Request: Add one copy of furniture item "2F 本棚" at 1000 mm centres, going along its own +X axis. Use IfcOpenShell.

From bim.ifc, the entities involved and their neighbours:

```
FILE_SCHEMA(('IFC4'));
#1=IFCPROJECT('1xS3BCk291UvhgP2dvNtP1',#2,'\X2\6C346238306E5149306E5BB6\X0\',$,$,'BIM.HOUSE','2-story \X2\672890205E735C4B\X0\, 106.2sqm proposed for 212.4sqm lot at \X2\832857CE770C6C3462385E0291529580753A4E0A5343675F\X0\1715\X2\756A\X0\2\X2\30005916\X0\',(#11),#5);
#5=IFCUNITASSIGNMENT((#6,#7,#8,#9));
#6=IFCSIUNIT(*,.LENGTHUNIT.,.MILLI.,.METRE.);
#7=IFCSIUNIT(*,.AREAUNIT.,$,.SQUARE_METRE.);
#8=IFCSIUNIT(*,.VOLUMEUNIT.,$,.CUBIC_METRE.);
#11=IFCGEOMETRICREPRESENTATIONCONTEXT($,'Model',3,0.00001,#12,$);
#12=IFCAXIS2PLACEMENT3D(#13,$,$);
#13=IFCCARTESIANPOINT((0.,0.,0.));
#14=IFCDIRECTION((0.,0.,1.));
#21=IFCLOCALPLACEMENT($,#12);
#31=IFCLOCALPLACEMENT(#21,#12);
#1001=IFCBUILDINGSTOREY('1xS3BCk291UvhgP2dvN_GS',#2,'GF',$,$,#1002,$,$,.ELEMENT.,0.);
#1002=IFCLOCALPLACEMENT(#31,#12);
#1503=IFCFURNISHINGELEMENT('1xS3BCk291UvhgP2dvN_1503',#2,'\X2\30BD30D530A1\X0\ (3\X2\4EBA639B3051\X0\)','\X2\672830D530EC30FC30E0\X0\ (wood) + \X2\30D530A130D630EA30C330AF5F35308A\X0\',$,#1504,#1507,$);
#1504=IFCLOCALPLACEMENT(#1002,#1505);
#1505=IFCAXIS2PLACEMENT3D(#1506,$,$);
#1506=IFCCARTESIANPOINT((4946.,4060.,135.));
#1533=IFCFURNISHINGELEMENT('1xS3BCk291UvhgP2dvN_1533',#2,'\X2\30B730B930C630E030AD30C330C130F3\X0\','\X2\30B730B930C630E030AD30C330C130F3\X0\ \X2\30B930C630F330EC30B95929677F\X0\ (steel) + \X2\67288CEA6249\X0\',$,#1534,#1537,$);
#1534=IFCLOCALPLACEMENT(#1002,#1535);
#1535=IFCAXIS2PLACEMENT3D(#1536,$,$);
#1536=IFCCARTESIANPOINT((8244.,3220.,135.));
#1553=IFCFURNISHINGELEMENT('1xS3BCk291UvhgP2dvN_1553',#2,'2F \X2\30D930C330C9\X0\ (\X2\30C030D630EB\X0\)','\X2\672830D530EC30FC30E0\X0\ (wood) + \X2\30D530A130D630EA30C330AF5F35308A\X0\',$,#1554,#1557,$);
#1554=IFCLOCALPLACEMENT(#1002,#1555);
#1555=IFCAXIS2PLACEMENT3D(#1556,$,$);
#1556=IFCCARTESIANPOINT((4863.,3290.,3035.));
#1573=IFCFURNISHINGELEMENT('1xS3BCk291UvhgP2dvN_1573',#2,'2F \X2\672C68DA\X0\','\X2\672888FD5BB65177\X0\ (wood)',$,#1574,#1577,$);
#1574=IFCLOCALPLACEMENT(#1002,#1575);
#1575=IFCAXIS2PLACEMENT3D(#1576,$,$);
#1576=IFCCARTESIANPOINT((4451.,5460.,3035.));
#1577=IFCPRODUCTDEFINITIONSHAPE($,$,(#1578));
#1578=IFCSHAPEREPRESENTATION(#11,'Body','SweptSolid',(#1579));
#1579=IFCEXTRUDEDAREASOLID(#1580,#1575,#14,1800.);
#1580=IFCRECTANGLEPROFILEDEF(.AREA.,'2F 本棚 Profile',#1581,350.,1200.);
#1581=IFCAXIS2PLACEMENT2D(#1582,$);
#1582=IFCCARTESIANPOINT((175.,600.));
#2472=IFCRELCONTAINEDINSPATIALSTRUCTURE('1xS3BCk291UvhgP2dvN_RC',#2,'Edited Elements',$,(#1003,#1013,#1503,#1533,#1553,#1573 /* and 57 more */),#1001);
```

```python
import ifcopenshell
import ifcopenshell.api.geometry
import ifcopenshell.api.root
import ifcopenshell.util.element
import ifcopenshell.util.placement

model = ifcopenshell.open("bim.ifc")


def reuse_history(source, copy):
    """copy_class also copies each property set's owner history, people and application; keep the originals."""
    for rel in copy.IsDefinedBy:
        if rel.is_a("IfcRelDefinesByProperties") and (history := rel.RelatingPropertyDefinition.OwnerHistory):
            rel.RelatingPropertyDefinition.OwnerHistory = source.OwnerHistory
            ifcopenshell.util.element.remove_deep2(model, history)


source = model.by_guid("1xS3BCk291UvhgP2dvN_1573")
base = ifcopenshell.util.placement.get_local_placement(source.ObjectPlacement)
step = base[:3, 0] * 1000.0

for i in range(1, 2):
    copy = ifcopenshell.api.root.copy_class(model, product=source)
    copy.Representation = ifcopenshell.util.element.copy_deep(
        model, source.Representation, exclude=["IfcGeometricRepresentationContext", "IfcRepresentationMap"]
    )
    reuse_history(source, copy)
    matrix = base.copy()
    matrix[:3, 3] += i * step
    print("added at", matrix[:3, 3].round(3) + 0.0)
    ifcopenshell.api.geometry.edit_object_placement(model, product=copy, matrix=matrix, is_si=False)

model.write("bim_updated.ifc")
```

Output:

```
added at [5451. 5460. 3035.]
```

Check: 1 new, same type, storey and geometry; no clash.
